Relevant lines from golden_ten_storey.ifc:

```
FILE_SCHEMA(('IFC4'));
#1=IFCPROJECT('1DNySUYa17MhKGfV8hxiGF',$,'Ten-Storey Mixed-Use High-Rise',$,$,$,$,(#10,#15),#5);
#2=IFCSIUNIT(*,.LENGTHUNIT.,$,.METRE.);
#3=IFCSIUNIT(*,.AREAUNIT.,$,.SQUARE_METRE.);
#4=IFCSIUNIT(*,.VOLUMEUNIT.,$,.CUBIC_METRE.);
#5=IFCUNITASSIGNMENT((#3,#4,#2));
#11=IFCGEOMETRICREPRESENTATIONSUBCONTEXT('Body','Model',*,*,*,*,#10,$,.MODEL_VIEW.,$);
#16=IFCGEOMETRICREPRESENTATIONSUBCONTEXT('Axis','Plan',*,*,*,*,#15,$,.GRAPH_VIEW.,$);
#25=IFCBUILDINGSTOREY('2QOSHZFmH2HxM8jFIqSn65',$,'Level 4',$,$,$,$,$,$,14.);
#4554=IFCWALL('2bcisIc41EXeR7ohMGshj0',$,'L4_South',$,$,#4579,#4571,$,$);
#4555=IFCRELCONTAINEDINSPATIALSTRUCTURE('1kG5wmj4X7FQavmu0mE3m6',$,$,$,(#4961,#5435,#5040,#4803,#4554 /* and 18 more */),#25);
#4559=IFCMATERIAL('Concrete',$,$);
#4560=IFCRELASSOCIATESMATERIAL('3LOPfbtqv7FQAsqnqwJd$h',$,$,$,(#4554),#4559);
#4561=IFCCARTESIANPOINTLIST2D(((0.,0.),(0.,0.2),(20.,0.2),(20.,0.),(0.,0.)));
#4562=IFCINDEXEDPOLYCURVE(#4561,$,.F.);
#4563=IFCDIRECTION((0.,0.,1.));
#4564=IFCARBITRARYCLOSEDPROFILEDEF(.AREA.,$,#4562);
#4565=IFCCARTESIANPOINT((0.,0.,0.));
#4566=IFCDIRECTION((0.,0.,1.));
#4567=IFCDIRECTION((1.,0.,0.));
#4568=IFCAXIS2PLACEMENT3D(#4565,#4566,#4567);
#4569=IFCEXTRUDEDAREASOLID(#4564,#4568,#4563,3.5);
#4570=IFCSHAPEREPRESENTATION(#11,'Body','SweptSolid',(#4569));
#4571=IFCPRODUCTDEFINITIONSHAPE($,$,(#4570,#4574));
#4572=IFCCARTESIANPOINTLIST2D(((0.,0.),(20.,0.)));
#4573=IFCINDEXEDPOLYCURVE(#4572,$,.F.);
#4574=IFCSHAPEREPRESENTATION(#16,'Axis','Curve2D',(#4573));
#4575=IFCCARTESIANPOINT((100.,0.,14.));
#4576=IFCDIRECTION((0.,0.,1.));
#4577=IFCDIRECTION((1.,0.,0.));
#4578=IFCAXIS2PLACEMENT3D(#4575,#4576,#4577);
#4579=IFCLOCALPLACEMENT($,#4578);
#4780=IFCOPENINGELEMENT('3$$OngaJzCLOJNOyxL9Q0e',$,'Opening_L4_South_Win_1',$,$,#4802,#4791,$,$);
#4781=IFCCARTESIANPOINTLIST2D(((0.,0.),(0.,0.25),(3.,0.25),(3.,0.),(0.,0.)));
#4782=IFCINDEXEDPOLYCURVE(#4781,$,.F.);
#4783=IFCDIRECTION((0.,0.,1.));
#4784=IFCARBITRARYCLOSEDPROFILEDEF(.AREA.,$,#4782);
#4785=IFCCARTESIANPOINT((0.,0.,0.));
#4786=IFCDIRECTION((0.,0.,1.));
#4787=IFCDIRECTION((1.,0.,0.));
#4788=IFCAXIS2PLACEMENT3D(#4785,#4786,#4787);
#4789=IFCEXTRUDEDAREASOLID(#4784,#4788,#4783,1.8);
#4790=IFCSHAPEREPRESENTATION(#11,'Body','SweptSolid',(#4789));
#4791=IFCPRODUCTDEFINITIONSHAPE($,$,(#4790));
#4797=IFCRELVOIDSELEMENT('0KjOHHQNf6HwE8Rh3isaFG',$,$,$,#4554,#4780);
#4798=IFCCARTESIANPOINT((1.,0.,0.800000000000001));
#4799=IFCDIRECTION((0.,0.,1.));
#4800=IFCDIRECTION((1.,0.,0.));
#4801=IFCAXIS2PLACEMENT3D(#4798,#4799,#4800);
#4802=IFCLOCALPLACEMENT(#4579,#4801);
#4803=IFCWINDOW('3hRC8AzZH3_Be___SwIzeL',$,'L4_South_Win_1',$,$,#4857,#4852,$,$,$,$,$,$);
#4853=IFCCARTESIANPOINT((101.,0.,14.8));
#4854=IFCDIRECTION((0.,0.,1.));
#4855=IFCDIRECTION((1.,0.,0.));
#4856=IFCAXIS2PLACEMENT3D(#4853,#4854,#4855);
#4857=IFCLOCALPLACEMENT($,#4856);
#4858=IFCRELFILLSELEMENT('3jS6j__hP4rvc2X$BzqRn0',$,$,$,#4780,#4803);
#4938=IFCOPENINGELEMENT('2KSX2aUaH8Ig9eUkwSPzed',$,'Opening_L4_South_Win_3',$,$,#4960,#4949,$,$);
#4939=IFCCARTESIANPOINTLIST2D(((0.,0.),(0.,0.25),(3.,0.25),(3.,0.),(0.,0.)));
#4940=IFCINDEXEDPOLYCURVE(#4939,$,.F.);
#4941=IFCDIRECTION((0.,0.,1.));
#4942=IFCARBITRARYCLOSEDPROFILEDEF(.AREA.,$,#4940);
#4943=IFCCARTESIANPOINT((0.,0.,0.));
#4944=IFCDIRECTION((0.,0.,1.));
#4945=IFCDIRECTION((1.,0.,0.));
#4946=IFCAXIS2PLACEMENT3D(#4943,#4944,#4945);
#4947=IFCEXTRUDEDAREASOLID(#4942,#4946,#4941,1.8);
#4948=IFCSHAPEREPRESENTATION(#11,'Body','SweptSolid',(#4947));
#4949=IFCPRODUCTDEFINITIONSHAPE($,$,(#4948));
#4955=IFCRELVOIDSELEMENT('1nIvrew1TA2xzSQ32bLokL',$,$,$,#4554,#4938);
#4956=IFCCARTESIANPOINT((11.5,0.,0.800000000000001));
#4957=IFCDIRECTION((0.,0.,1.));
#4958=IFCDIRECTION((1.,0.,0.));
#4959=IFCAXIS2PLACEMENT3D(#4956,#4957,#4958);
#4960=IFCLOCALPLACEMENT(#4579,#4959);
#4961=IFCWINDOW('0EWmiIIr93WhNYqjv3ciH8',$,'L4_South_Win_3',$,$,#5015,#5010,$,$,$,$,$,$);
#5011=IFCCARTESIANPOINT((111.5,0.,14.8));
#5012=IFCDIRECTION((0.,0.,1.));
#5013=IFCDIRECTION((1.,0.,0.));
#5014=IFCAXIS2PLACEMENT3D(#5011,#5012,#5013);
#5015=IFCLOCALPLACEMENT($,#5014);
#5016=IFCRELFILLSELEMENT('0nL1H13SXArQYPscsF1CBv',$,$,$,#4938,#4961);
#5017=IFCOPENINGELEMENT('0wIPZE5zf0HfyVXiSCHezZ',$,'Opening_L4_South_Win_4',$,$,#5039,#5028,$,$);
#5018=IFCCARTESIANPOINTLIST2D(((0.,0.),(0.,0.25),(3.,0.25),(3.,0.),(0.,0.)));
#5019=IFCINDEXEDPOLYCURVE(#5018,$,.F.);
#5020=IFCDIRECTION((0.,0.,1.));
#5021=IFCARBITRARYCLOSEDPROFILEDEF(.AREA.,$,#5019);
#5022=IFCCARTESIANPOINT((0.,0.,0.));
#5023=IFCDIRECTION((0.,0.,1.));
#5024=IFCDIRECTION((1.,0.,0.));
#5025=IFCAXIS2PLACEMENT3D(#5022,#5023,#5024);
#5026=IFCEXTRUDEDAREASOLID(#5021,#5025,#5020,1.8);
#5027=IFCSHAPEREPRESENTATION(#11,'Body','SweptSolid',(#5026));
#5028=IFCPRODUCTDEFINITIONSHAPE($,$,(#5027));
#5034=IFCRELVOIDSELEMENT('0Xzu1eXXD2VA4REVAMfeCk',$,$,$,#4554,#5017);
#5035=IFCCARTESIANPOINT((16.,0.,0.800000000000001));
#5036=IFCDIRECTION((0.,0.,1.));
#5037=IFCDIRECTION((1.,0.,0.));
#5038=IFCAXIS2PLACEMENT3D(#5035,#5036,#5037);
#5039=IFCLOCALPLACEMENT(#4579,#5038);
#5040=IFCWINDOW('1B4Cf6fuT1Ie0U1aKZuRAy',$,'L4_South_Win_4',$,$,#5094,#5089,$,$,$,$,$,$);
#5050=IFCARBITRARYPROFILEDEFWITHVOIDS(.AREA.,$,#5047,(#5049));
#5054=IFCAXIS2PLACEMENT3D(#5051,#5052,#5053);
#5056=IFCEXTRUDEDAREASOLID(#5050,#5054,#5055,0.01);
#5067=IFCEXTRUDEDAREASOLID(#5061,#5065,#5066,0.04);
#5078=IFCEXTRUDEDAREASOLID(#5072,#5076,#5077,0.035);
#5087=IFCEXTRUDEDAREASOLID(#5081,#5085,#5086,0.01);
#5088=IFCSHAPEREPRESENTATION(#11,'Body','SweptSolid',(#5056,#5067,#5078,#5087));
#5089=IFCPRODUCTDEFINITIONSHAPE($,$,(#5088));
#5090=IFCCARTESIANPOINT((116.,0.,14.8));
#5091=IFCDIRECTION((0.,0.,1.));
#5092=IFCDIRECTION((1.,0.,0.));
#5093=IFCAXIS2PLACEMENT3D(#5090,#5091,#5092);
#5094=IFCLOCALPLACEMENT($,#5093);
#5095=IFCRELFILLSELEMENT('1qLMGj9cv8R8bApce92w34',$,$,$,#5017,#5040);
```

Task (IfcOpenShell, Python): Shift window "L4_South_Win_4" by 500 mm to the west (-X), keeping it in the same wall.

```python
import ifcopenshell
import ifcopenshell.api.geometry
import ifcopenshell.util.placement
import ifcopenshell.util.unit

model = ifcopenshell.open("golden_ten_storey.ifc")
unit_scale = ifcopenshell.util.unit.calculate_unit_scale(model)

window = model.by_id(5040)
opening = window.FillsVoids[0].RelatingOpeningElement
wall = opening.VoidsElements[0].RelatingBuildingElement

wall_matrix = ifcopenshell.util.placement.get_local_placement(wall.ObjectPlacement)
shift = wall_matrix[:3, 0] * -0.5 / unit_scale
before = ifcopenshell.util.placement.get_local_placement(window.ObjectPlacement)[:3, 3].copy()

# The window is not placed relative to its opening, so move both.
for product in (opening, window):
    matrix = ifcopenshell.util.placement.get_local_placement(product.ObjectPlacement)
    matrix[:3, 3] += shift
    ifcopenshell.api.geometry.edit_object_placement(model, product=product, matrix=matrix, is_si=False)

after = ifcopenshell.util.placement.get_local_placement(window.ObjectPlacement)[:3, 3]
print("window moved by", (after - before).round(3) + 0.0)

model.write("golden_ten_storey_v2.ifc")
```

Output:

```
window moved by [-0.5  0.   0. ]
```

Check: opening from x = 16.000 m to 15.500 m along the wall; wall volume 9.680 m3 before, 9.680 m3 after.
